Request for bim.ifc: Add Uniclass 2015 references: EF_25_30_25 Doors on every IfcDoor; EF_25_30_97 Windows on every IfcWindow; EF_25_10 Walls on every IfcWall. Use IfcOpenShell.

First a look at what the model holds.

```python
import ifcopenshell

model = ifcopenshell.open("bim.ifc")
print(model.schema)
print("classifications:", [c.Name for c in model.by_type("IfcClassification")])
for ifc_class in ("IfcDoor", "IfcRoof", "IfcStair", "IfcWall", "IfcWindow"):
    print(ifc_class, len(model.by_type(ifc_class)))
```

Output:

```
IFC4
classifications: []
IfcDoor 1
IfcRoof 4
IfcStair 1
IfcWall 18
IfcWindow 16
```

```python
import ifcopenshell
import ifcopenshell.api.classification

model = ifcopenshell.open("bim.ifc")

system = ifcopenshell.api.classification.add_classification(model, classification="Uniclass 2015")

codes = {
    "IfcDoor": ("EF_25_30_25", "Doors"),
    "IfcWindow": ("EF_25_30_97", "Windows"),
    "IfcWall": ("EF_25_10", "Walls"),
}
for ifc_class, (code, name) in codes.items():
    products = model.by_type(ifc_class)
    ifcopenshell.api.classification.add_reference(
        model, products=products, classification=system, identification=code, name=name
    )
    print(code, len(products))

model.write("bim-out.ifc")
```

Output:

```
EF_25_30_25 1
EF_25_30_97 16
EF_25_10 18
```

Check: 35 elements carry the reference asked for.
